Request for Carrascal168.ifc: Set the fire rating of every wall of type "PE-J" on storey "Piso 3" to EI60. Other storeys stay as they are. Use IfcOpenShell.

First a look at what the model holds.

```python
import ifcopenshell
import ifcopenshell.util.element

model = ifcopenshell.open("Carrascal168.ifc")
print(model.schema)
storey = next(s for s in model.by_type("IfcBuildingStorey") if s.Name == "Piso 3")
walls = [e for e in ifcopenshell.util.element.get_decomposition(storey) if e.is_a("IfcWall")]
seen = {}
for e in walls:
    element_type = ifcopenshell.util.element.get_type(e)
    key = (element_type.Name if element_type != e and element_type else None, ifcopenshell.util.element.get_pset(e, "Pset_WallCommon", "FireRating"))
    seen[key] = seen.get(key, 0) + 1
for (name, value), count in sorted(seen.items(), key=str):
    print(count, "x", name, "|", value)
```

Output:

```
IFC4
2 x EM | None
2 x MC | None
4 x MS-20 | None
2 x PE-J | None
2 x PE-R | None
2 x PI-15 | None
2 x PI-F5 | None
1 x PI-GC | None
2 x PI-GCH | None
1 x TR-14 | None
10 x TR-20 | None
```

```python
import ifcopenshell
import ifcopenshell.api.pset
import ifcopenshell.util.element

model = ifcopenshell.open("Carrascal168.ifc")

storey = next(s for s in model.by_type("IfcBuildingStorey") if s.Name == "Piso 3")
walls = [e for e in ifcopenshell.util.element.get_decomposition(storey) if e.is_a("IfcWall")]

count = 0
for e in walls:
    element_type = ifcopenshell.util.element.get_type(e)
    if element_type in (None, e) or element_type.Name != "PE-J":
        continue
    # add_pset returns the element's existing set when there is one.
    pset = ifcopenshell.api.pset.add_pset(model, product=e, name="Pset_WallCommon")
    ifcopenshell.api.pset.edit_pset(model, pset=pset, properties={"FireRating": "EI60"})
    count += 1

print(count, "walls updated")

model.write("Carrascal168_v2.ifc")
```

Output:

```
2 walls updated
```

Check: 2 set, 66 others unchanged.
